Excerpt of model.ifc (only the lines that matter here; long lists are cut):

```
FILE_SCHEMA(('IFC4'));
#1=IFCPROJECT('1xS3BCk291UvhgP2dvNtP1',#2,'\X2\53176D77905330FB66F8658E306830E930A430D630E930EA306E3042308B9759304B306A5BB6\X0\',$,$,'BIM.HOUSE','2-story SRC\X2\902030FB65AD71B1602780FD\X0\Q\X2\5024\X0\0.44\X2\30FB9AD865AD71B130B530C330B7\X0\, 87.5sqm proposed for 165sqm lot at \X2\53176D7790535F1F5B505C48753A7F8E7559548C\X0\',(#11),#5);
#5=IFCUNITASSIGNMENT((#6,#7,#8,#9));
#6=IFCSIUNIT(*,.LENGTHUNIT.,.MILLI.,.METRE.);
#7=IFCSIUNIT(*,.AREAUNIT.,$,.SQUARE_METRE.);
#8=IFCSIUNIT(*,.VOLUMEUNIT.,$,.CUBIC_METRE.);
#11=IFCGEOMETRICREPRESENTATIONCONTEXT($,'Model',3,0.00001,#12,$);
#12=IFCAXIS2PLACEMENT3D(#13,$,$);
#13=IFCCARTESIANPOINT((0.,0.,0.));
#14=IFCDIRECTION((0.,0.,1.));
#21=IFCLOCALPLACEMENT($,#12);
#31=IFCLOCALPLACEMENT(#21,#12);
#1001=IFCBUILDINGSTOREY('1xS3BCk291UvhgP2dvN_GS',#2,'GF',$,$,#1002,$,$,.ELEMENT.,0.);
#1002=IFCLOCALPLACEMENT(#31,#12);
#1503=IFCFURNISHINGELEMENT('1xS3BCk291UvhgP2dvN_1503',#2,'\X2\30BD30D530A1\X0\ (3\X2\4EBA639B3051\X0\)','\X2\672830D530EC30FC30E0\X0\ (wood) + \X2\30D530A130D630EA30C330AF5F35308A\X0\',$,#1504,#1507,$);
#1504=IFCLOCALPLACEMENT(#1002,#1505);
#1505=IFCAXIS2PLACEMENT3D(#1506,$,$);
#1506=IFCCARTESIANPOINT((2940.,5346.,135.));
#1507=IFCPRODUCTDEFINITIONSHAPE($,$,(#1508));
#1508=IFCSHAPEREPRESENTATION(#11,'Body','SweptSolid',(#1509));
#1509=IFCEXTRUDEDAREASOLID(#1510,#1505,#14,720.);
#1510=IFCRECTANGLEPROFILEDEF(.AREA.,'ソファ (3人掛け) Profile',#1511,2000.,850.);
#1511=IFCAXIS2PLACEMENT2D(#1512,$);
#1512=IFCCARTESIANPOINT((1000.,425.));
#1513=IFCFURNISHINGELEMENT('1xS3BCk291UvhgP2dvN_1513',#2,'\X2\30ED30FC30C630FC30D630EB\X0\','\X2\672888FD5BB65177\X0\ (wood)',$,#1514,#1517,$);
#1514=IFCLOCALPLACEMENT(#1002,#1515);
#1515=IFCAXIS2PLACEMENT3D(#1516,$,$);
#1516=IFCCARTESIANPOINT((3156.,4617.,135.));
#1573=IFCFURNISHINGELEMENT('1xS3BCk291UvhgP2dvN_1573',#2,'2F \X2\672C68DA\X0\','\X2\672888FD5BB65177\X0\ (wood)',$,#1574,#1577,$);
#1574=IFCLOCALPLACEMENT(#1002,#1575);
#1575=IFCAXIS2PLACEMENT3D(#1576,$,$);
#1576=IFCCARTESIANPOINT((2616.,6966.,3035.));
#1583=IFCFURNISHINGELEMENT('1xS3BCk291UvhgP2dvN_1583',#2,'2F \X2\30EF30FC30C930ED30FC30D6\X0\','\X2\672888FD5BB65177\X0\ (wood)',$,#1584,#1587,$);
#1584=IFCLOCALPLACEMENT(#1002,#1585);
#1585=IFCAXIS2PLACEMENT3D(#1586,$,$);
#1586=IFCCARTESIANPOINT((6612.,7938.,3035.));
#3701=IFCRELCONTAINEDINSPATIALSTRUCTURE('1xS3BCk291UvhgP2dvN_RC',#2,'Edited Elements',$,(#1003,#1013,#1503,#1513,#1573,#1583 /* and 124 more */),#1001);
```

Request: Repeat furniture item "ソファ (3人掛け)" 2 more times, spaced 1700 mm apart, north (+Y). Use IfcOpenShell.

```python
import numpy as np
import ifcopenshell
import ifcopenshell.api.geometry
import ifcopenshell.api.root
import ifcopenshell.util.element
import ifcopenshell.util.placement
import ifcopenshell.util.unit

model = ifcopenshell.open("model.ifc")
unit_scale = ifcopenshell.util.unit.calculate_unit_scale(model)


def reuse_history(source, copy):
    """copy_class also copies each property set's owner history, people and application; keep the originals."""
    for rel in copy.IsDefinedBy:
        if rel.is_a("IfcRelDefinesByProperties") and (history := rel.RelatingPropertyDefinition.OwnerHistory):
            rel.RelatingPropertyDefinition.OwnerHistory = source.OwnerHistory
            ifcopenshell.util.element.remove_deep2(model, history)


source = model.by_guid("1xS3BCk291UvhgP2dvN_1503")
base = ifcopenshell.util.placement.get_local_placement(source.ObjectPlacement)
step = np.array([0.0, 1.0, 0.0]) * 1.7 / unit_scale

for i in range(1, 3):
    copy = ifcopenshell.api.root.copy_class(model, product=source)
    copy.Representation = ifcopenshell.util.element.copy_deep(
        model, source.Representation, exclude=["IfcGeometricRepresentationContext", "IfcRepresentationMap"]
    )
    reuse_history(source, copy)
    matrix = base.copy()
    matrix[:3, 3] += i * step
    print("added at", matrix[:3, 3].round(3) + 0.0)
    ifcopenshell.api.geometry.edit_object_placement(model, product=copy, matrix=matrix, is_si=False)

model.write("model_edited.ifc")
```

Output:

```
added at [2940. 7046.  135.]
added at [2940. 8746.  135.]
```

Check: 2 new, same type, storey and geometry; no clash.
